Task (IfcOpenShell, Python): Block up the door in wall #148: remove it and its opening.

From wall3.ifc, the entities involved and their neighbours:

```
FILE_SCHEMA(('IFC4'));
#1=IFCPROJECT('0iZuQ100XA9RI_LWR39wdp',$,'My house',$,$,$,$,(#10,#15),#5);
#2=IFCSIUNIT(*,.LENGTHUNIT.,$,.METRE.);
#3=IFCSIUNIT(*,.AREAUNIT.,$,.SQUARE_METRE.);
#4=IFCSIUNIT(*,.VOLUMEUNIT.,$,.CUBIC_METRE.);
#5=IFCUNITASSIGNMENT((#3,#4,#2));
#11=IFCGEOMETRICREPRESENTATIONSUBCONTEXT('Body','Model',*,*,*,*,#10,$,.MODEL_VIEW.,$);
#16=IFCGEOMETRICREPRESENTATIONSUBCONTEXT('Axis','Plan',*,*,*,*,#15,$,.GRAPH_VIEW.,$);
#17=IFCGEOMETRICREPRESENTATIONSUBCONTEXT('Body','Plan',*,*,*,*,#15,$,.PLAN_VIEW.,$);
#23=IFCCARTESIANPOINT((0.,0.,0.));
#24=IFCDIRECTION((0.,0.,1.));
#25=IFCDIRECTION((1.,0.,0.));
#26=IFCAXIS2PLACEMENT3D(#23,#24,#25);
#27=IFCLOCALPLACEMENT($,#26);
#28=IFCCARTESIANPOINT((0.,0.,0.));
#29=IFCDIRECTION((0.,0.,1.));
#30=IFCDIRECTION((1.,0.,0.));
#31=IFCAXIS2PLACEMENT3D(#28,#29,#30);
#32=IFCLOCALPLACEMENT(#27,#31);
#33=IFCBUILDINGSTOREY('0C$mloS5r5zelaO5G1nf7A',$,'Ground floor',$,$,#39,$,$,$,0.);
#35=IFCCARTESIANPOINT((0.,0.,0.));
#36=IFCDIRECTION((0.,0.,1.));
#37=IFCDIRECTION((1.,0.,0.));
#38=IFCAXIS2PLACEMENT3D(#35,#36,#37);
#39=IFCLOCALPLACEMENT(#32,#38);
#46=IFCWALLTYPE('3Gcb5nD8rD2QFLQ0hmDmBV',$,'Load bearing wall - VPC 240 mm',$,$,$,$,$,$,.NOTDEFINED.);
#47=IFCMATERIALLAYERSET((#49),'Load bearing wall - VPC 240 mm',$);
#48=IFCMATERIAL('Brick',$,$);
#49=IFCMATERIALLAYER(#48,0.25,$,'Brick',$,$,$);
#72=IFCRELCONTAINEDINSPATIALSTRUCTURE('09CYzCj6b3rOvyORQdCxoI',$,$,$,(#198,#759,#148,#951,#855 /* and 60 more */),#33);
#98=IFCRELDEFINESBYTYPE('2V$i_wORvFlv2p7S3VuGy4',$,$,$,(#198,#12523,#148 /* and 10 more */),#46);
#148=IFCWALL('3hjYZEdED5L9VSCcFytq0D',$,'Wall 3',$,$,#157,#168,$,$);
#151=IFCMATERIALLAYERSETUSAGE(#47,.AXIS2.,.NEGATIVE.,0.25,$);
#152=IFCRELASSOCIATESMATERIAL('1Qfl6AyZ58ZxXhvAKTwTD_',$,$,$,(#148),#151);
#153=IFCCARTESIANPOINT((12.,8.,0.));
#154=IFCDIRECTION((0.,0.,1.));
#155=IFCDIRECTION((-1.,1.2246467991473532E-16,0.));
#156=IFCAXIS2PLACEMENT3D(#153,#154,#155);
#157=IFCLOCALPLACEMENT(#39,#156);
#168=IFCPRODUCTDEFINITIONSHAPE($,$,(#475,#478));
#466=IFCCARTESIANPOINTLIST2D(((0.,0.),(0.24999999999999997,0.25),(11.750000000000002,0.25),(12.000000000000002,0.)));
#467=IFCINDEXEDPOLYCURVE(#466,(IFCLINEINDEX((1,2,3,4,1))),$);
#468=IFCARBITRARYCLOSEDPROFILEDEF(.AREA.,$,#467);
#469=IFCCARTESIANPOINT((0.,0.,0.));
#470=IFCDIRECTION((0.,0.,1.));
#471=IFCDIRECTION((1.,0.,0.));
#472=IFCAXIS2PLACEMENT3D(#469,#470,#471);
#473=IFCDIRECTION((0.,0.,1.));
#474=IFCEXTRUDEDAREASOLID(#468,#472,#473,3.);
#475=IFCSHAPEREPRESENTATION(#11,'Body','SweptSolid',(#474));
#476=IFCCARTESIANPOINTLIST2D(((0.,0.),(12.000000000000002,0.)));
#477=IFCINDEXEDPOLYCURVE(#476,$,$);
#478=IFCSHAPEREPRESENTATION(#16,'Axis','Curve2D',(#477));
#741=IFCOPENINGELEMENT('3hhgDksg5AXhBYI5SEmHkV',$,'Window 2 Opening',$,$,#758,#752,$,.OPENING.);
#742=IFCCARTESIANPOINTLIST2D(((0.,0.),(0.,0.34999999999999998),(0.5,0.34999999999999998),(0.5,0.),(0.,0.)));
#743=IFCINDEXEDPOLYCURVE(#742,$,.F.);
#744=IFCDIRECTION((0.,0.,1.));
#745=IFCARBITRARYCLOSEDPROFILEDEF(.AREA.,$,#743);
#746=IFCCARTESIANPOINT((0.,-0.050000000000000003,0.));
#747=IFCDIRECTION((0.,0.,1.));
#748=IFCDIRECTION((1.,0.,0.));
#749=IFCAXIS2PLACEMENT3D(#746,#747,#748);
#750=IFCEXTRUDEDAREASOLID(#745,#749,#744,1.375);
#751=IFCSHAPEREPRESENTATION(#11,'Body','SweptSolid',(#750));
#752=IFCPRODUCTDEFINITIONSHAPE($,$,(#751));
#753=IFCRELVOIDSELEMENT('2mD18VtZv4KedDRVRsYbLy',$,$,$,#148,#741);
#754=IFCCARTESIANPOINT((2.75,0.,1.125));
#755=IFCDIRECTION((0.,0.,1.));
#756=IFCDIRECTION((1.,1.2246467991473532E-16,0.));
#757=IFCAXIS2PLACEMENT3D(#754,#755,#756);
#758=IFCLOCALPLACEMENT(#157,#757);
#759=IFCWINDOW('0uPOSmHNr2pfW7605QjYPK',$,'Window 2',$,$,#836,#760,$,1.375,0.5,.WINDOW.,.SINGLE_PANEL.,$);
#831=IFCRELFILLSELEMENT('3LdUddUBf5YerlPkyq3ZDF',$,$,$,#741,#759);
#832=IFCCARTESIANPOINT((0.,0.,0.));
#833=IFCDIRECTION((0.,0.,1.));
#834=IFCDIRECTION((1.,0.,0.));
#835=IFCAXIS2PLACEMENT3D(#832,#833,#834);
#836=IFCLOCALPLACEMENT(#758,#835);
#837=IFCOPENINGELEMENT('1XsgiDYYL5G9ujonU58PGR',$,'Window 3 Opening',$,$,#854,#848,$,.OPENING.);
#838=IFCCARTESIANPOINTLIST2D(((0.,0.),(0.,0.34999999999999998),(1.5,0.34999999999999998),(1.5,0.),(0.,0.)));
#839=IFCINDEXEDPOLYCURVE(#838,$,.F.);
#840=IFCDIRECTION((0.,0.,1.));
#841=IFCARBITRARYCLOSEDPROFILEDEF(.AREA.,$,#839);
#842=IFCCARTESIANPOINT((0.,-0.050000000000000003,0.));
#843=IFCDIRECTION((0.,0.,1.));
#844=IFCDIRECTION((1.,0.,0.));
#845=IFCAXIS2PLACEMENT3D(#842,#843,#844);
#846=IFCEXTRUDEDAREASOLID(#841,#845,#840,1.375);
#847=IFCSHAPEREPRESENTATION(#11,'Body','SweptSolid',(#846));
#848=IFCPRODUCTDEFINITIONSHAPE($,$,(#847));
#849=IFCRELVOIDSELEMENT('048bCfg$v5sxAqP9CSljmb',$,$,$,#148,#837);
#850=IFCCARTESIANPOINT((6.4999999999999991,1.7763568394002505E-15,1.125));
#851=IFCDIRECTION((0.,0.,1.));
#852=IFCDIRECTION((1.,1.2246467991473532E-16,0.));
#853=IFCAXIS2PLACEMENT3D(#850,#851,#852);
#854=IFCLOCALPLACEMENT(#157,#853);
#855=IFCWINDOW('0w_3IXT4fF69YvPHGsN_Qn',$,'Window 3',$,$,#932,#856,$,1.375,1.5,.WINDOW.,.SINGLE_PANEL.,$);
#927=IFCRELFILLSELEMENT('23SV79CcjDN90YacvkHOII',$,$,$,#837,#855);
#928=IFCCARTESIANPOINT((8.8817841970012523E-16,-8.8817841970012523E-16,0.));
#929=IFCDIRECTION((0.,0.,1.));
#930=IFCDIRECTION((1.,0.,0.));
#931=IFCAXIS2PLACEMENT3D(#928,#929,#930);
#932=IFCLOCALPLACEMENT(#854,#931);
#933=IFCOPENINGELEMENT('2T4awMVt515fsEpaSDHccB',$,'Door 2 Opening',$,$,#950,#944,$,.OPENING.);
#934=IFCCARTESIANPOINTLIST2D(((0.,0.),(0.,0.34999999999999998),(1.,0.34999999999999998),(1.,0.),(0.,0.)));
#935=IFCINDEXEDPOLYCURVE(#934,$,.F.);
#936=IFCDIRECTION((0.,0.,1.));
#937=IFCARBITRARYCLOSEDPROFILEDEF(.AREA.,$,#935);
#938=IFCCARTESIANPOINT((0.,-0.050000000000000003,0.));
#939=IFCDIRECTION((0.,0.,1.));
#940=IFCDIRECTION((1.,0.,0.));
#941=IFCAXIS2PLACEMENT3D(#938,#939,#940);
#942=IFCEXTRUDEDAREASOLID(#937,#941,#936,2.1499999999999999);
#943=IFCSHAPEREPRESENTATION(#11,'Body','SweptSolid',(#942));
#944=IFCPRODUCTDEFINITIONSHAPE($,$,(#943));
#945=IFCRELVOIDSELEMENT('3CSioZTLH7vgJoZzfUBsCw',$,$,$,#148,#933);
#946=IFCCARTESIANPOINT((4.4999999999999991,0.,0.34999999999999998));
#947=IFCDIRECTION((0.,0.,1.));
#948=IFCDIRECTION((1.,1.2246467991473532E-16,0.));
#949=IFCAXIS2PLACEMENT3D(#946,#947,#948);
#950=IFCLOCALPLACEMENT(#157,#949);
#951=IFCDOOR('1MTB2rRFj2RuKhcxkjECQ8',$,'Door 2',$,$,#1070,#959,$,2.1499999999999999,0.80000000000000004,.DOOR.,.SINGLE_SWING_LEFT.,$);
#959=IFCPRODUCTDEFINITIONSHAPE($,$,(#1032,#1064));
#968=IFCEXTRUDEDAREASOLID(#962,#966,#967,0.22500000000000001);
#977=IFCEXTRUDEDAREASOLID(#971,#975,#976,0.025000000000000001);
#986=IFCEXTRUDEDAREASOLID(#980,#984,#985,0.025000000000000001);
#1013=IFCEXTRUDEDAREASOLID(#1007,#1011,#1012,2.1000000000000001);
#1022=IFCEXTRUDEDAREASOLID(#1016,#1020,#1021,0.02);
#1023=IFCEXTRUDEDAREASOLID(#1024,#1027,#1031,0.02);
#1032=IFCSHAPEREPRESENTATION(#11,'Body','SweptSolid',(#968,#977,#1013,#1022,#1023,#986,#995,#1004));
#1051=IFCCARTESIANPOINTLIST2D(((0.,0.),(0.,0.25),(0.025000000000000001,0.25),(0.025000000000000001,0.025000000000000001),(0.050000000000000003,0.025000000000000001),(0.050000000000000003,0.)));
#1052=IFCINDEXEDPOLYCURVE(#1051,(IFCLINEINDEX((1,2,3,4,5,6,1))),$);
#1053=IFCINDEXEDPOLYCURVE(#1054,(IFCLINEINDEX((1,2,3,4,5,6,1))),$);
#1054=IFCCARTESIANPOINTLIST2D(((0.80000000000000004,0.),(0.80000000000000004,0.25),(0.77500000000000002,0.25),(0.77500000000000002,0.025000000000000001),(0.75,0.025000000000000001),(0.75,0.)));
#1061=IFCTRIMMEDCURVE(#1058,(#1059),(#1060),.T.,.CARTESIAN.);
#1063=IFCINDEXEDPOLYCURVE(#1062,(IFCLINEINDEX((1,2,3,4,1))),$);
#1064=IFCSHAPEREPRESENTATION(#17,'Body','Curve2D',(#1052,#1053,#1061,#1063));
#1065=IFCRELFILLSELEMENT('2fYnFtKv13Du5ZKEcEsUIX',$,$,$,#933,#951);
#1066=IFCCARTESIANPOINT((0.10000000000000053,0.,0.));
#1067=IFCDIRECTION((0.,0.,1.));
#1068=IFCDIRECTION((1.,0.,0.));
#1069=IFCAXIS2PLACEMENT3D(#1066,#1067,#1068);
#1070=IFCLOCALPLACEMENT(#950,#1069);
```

```python
import ifcopenshell
import ifcopenshell.api.feature
import ifcopenshell.api.root
import ifcopenshell.geom
import ifcopenshell.util.shape

model = ifcopenshell.open("wall3.ifc")
settings = ifcopenshell.geom.settings()


def volume(element):
    """Net volume in cubic metres, openings subtracted."""
    shape = ifcopenshell.geom.create_shape(settings, element)
    return ifcopenshell.util.shape.get_volume(shape.geometry)


door = model.by_id(951)
opening = door.FillsVoids[0].RelatingOpeningElement
wall = opening.VoidsElements[0].RelatingBuildingElement
before = volume(wall)

ifcopenshell.api.root.remove_product(model, product=door)
ifcopenshell.api.feature.remove_feature(model, feature=opening)

after = volume(wall)

print(f"wall volume {before:.3f} -> {after:.3f} m3")

model.write("wall3_edited.ifc")
```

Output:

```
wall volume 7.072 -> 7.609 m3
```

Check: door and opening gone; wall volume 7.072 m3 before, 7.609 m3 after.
